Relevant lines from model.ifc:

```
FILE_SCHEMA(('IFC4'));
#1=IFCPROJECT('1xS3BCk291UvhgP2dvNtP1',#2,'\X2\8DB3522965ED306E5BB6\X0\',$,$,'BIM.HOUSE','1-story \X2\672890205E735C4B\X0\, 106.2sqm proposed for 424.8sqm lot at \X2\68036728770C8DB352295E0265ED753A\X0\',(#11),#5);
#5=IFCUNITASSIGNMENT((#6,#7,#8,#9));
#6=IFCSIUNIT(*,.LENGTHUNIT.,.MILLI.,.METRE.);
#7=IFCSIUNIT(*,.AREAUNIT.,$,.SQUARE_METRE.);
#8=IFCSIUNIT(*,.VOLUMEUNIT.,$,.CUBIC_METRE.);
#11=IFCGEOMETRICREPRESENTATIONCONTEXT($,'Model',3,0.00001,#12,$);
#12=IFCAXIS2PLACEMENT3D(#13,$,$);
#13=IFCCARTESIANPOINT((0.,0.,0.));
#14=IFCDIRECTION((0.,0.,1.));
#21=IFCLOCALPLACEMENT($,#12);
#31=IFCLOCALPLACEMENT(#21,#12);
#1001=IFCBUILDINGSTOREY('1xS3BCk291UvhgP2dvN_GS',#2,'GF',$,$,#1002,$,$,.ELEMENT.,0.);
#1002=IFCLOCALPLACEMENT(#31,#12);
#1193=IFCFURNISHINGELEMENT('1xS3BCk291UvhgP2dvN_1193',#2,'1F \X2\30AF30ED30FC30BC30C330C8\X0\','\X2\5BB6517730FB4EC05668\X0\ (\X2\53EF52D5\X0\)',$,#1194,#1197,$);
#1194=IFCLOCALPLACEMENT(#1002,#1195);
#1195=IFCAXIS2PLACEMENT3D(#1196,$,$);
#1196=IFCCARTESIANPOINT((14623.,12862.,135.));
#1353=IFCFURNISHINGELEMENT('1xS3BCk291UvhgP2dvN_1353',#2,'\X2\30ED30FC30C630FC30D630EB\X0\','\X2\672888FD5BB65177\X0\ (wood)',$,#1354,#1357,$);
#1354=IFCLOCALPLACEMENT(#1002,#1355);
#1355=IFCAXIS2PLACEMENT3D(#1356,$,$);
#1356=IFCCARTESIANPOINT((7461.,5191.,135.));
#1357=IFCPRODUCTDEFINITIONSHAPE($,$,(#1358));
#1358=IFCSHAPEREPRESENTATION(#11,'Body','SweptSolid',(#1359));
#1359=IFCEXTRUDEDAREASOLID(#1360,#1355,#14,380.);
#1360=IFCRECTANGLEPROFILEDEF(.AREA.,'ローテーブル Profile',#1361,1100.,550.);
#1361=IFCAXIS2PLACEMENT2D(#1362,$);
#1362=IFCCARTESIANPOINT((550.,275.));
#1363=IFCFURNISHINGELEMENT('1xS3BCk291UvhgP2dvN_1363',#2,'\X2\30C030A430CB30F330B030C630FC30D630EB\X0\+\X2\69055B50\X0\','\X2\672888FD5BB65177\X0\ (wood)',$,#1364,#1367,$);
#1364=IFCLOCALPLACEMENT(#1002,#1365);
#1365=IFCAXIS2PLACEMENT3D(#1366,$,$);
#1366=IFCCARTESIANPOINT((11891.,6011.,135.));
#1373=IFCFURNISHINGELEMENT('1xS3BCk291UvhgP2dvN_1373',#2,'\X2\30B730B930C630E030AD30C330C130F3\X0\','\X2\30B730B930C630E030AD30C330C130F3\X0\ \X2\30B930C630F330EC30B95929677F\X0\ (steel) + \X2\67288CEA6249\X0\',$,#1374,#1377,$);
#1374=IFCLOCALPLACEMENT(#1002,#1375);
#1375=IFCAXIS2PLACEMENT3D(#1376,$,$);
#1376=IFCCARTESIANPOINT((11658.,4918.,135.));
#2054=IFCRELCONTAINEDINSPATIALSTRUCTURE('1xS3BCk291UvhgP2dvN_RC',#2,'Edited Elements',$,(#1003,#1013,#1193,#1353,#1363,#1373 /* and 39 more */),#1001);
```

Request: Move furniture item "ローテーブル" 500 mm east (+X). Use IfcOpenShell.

```python
import ifcopenshell
import ifcopenshell.api.geometry
import ifcopenshell.util.placement
import ifcopenshell.util.unit

model = ifcopenshell.open("model.ifc")
unit_scale = ifcopenshell.util.unit.calculate_unit_scale(model)

item = model.by_id(1353)
matrix = ifcopenshell.util.placement.get_local_placement(item.ObjectPlacement)
matrix[0, 3] += 0.5 / unit_scale
ifcopenshell.api.geometry.edit_object_placement(model, product=item, matrix=matrix, is_si=False)

print(ifcopenshell.util.placement.get_local_placement(item.ObjectPlacement).round(3) + 0.0)

model.write("model_edited.ifc")
```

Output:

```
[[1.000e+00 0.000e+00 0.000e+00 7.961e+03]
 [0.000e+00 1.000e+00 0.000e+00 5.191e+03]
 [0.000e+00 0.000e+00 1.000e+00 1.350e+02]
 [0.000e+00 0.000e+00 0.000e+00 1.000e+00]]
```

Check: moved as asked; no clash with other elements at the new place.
